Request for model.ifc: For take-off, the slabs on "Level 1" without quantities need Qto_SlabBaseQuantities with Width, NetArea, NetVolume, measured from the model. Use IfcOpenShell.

First a look at what the model holds.

```python
import ifcopenshell
import ifcopenshell.util.element
import ifcopenshell.util.unit

model = ifcopenshell.open("model.ifc")
print(model.schema)
for unit_type in ("LENGTHUNIT", "AREAUNIT", "VOLUMEUNIT"):
    print(unit_type, ifcopenshell.util.unit.calculate_unit_scale(model, unit_type))
storey = next(s for s in model.by_type("IfcBuildingStorey") if s.Name == "Level 1")
slabs = [e for e in ifcopenshell.util.element.get_decomposition(storey) if e.is_a("IfcSlab")]
for e in sorted(slabs, key=lambda e: e.id()):
    print(e.id(), e.is_a(), e.Name, list(ifcopenshell.util.element.get_psets(e, qtos_only=True)), sep=" | ")
```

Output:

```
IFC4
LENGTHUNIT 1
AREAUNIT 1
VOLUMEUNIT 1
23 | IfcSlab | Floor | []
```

```python
import ifcopenshell
import ifcopenshell.api.pset
import ifcopenshell.geom
import ifcopenshell.util.element
import ifcopenshell.util.shape
import ifcopenshell.util.unit

model = ifcopenshell.open("model.ifc")
unit_scale = ifcopenshell.util.unit.calculate_unit_scale(model)
area_scale = ifcopenshell.util.unit.calculate_unit_scale(model, "AREAUNIT")
volume_scale = ifcopenshell.util.unit.calculate_unit_scale(model, "VOLUMEUNIT")
settings = ifcopenshell.geom.settings()

storey = next(s for s in model.by_type("IfcBuildingStorey") if s.Name == "Level 1")
slabs = [e for e in ifcopenshell.util.element.get_decomposition(storey) if e.is_a("IfcSlab")]

for e in sorted(slabs, key=lambda e: e.id()):
    if ifcopenshell.util.element.get_psets(e, qtos_only=True, should_inherit=False):
        continue
    # Geometry comes back in metres, in the element's own axes.
    shape = ifcopenshell.geom.create_shape(settings, e)
    values = {
        "Width": ifcopenshell.util.shape.get_z(shape.geometry) / unit_scale,
        "NetArea": ifcopenshell.util.shape.get_footprint_area(shape.geometry) / area_scale,
        "NetVolume": ifcopenshell.util.shape.get_volume(shape.geometry) / volume_scale,
    }
    qto = ifcopenshell.api.pset.add_qto(model, product=e, name="Qto_SlabBaseQuantities")
    ifcopenshell.api.pset.edit_qto(model, qto=qto, properties=values)
    print(e.id(), {k: round(v, 3) for k, v in values.items()})

model.write("model_edited.ifc")
```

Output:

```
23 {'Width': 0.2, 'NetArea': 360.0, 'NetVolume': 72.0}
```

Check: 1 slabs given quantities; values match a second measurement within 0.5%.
